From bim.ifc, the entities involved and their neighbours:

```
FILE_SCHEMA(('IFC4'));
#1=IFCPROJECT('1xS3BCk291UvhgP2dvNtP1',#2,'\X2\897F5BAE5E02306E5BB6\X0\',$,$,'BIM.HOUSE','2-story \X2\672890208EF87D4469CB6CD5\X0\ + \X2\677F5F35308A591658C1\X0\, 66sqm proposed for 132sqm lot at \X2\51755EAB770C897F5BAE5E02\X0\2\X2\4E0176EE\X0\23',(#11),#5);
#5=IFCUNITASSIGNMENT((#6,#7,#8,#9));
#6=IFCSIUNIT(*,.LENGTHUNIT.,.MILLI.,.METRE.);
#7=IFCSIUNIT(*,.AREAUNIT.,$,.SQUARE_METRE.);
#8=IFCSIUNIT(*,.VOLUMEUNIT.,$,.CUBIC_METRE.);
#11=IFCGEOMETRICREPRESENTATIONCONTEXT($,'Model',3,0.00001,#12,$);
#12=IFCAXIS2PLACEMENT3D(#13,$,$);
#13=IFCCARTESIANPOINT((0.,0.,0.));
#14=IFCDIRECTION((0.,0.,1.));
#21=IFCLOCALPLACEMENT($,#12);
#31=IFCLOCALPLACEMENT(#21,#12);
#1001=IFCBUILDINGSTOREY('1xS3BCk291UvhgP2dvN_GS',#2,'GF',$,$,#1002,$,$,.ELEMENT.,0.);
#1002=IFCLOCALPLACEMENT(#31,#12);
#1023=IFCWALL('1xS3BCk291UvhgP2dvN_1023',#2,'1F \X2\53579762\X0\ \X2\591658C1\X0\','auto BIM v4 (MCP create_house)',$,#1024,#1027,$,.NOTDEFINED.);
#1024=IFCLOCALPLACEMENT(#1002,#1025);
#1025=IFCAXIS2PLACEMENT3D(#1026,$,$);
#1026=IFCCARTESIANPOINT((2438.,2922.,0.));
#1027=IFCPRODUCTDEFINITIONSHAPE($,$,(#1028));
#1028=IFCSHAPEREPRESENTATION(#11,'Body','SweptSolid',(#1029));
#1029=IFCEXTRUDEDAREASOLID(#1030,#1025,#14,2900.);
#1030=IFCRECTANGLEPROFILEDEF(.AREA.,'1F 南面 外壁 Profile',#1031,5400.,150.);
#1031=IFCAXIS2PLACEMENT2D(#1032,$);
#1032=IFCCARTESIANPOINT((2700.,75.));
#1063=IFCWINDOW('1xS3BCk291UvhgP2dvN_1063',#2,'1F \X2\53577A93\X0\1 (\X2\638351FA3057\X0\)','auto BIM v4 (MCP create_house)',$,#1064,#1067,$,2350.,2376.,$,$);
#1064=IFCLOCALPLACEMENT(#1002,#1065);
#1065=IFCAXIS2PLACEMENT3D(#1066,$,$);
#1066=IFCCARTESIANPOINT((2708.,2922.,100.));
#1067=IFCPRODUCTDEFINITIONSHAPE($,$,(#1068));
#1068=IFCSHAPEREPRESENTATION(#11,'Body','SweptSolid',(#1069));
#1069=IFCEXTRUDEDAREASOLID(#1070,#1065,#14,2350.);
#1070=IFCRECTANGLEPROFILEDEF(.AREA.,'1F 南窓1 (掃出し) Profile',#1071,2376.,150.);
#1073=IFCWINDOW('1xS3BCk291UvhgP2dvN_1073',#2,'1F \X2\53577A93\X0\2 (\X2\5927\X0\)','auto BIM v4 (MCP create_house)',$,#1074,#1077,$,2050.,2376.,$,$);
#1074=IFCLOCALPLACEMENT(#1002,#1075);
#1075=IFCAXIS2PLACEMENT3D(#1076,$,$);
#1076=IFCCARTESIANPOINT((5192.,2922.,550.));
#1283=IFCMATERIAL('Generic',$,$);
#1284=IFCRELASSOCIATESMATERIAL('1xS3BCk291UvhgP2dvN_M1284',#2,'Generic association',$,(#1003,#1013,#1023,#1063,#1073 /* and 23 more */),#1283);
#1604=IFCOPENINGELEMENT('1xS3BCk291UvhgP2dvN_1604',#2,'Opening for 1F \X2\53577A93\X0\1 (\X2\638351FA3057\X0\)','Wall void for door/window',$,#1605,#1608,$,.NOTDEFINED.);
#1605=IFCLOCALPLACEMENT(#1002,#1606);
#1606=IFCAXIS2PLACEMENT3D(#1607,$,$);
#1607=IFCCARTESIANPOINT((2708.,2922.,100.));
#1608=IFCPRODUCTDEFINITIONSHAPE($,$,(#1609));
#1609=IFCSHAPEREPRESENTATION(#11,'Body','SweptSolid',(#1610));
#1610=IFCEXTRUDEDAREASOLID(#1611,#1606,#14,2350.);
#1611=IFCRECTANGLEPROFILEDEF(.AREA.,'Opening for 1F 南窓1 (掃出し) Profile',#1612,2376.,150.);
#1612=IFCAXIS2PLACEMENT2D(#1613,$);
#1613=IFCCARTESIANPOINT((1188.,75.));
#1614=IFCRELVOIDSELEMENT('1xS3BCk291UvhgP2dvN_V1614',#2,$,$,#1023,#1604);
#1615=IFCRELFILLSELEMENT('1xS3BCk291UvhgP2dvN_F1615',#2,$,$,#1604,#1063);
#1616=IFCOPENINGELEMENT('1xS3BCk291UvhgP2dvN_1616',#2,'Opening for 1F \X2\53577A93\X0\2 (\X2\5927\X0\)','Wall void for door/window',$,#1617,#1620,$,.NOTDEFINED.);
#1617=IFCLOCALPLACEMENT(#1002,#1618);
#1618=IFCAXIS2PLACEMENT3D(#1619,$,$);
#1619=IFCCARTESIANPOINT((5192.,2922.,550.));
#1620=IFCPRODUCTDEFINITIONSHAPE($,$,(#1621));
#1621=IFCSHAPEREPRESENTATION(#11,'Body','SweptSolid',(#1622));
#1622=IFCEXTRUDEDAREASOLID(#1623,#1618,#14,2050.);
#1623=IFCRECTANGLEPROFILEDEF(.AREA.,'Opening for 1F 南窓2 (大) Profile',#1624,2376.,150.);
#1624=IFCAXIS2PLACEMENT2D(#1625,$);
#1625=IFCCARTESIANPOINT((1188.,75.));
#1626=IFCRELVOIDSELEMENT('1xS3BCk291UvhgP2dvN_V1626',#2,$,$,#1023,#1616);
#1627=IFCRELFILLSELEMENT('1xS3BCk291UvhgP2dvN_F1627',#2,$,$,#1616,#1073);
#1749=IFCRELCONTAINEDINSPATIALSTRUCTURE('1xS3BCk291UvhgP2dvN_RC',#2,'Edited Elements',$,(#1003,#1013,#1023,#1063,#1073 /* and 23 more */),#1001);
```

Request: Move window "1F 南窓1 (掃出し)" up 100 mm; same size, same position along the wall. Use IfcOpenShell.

```python
import numpy as np
import ifcopenshell
import ifcopenshell.api.geometry
import ifcopenshell.util.placement
import ifcopenshell.util.unit

model = ifcopenshell.open("bim.ifc")
unit_scale = ifcopenshell.util.unit.calculate_unit_scale(model)

window = model.by_id(1063)
opening = window.FillsVoids[0].RelatingOpeningElement
dz = 0.1 / unit_scale

shift = np.array([0.0, 0.0, dz])
# The window is not placed relative to its opening, so move both.
for product in (opening, window):
    matrix = ifcopenshell.util.placement.get_local_placement(product.ObjectPlacement)
    matrix[:3, 3] += shift
    ifcopenshell.api.geometry.edit_object_placement(model, product=product, matrix=matrix, is_si=False)

print(f"moved by {dz * unit_scale:+.3f} m")

model.write("bim-out.ifc")
```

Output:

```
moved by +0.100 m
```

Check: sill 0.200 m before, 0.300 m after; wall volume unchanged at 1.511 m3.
